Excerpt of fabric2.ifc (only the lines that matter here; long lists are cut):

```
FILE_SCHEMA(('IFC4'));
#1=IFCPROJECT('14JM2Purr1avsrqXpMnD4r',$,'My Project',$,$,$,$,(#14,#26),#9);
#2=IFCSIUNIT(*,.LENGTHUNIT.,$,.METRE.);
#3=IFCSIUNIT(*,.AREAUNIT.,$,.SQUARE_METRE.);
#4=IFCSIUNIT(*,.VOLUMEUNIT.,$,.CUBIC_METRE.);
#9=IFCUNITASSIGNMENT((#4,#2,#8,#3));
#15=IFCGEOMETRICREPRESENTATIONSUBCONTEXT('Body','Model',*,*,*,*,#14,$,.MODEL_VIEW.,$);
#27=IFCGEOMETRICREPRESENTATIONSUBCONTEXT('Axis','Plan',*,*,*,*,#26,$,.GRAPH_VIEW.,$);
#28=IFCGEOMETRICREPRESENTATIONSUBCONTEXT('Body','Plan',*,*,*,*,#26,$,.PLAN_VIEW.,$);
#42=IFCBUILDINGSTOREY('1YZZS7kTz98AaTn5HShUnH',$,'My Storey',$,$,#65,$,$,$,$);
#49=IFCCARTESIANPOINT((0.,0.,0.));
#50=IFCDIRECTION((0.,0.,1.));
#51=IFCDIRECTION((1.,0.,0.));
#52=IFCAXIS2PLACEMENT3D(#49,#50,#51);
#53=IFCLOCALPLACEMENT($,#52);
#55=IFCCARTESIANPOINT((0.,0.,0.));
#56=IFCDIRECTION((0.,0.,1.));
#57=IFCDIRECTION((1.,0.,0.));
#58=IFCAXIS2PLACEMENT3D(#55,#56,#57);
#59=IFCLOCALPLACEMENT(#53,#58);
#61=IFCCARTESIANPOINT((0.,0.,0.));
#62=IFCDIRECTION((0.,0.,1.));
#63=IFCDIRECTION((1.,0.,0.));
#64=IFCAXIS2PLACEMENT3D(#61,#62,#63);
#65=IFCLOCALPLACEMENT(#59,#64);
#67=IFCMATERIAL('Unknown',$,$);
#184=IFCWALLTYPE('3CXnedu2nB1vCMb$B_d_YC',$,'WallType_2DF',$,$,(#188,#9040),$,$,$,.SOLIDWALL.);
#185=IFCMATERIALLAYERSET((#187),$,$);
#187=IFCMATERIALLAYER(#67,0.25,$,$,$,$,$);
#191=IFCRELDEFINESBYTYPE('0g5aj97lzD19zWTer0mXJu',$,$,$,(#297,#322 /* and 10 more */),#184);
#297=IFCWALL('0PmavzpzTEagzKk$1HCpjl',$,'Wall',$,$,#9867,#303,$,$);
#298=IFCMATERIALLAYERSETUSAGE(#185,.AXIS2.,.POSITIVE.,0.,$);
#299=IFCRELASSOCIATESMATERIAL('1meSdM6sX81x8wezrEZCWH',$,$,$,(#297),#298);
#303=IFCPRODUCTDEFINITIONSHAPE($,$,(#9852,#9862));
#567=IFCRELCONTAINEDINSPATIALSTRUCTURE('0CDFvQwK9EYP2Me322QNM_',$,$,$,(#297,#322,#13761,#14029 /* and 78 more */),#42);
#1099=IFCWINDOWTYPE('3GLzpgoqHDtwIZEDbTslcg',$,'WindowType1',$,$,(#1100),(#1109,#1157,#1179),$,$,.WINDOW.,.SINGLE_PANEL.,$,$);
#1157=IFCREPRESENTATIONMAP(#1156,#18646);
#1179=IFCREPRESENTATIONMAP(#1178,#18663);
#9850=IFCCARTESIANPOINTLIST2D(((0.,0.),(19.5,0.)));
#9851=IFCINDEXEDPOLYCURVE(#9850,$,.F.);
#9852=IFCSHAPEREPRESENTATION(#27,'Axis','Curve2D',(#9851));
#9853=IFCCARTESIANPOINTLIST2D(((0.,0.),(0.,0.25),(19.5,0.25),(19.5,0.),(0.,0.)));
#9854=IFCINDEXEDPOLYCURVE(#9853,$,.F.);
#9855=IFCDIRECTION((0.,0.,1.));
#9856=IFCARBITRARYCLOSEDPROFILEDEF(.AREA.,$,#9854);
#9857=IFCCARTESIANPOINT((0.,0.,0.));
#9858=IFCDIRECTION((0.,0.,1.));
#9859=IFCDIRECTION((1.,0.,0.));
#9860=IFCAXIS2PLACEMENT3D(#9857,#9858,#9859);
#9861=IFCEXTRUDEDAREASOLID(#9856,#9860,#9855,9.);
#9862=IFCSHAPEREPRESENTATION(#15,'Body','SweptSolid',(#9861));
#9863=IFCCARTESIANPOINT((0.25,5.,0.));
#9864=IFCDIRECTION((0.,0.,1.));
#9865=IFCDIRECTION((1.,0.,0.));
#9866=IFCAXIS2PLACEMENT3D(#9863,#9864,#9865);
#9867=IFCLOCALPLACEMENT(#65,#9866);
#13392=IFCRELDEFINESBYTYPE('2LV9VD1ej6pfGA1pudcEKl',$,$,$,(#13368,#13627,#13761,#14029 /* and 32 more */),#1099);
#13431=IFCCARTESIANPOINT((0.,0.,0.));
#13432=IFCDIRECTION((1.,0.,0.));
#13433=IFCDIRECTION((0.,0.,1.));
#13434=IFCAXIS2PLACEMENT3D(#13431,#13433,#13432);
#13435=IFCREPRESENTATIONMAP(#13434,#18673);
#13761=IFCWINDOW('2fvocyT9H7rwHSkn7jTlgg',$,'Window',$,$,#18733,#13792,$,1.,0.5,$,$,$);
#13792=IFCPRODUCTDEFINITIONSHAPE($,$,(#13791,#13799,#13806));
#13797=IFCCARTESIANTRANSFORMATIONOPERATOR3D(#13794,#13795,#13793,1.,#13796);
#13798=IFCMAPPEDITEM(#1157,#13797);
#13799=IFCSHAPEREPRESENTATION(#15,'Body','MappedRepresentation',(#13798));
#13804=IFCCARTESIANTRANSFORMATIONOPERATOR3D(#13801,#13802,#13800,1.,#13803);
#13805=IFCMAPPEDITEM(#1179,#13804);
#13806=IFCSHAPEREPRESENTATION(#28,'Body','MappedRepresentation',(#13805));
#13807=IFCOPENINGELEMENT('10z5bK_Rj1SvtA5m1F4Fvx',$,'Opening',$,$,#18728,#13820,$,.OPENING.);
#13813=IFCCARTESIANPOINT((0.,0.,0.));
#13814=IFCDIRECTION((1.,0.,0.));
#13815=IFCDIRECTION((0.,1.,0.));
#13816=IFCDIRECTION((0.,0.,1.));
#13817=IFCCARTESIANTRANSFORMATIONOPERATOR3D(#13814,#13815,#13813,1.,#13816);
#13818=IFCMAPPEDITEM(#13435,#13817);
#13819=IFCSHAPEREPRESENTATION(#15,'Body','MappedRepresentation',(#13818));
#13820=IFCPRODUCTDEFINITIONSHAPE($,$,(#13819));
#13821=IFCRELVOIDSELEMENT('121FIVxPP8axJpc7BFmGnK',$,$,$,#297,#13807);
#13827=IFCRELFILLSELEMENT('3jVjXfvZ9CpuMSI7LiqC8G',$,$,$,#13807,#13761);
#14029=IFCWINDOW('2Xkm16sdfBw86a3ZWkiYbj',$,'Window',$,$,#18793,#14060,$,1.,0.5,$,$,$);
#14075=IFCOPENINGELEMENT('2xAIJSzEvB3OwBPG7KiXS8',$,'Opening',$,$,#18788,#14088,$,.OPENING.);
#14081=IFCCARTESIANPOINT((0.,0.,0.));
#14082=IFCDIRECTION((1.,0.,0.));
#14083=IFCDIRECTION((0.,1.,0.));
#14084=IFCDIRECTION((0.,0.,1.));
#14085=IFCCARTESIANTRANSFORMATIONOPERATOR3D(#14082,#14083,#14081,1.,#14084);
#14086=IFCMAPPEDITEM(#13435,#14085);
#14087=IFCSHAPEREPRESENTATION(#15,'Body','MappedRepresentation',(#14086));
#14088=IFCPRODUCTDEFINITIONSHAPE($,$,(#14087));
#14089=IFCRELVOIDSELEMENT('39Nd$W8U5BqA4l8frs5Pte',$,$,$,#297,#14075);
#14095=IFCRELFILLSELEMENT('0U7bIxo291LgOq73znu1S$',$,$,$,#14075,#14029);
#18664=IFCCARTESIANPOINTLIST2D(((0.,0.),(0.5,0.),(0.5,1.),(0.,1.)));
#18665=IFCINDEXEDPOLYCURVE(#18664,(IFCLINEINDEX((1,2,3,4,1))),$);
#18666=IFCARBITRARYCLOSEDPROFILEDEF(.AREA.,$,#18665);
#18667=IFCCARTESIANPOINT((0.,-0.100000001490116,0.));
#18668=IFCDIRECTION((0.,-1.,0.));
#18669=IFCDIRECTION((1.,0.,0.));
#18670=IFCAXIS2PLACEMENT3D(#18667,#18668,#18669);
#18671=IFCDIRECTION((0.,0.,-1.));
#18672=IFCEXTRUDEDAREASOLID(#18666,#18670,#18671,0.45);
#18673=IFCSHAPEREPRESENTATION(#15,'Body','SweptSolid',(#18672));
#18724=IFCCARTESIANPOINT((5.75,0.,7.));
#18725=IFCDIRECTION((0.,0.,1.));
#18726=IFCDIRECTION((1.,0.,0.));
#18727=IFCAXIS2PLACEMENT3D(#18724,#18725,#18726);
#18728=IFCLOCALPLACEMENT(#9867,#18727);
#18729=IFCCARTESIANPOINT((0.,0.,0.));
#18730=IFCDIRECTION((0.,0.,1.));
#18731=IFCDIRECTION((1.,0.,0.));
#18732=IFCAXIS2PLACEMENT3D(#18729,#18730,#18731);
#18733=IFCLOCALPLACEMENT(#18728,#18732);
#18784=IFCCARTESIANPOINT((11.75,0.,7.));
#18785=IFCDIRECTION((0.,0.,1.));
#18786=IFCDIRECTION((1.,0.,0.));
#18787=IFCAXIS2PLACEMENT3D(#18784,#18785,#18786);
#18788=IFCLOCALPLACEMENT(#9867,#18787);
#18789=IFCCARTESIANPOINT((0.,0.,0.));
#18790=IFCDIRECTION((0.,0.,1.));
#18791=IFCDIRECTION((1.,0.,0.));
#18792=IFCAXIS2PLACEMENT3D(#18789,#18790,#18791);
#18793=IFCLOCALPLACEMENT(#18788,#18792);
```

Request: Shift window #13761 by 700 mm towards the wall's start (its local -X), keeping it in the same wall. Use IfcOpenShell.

```python
import ifcopenshell
import ifcopenshell.api.geometry
import ifcopenshell.util.placement

model = ifcopenshell.open("fabric2.ifc")

window = model.by_guid("2fvocyT9H7rwHSkn7jTlgg")
opening = window.FillsVoids[0].RelatingOpeningElement
wall = opening.VoidsElements[0].RelatingBuildingElement

wall_matrix = ifcopenshell.util.placement.get_local_placement(wall.ObjectPlacement)
shift = wall_matrix[:3, 0] * -0.7
before = ifcopenshell.util.placement.get_local_placement(window.ObjectPlacement)[:3, 3].copy()

# The window is placed relative to its opening, so it follows when the opening moves.
matrix = ifcopenshell.util.placement.get_local_placement(opening.ObjectPlacement)
matrix[:3, 3] += shift
ifcopenshell.api.geometry.edit_object_placement(
    model, product=opening, matrix=matrix, is_si=False, should_transform_children=True
)

after = ifcopenshell.util.placement.get_local_placement(window.ObjectPlacement)[:3, 3]
print("window moved by", (after - before).round(3) + 0.0)

model.write("fabric2_v2.ifc")
```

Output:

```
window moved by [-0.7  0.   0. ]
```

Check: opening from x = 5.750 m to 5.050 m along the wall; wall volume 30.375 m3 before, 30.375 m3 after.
